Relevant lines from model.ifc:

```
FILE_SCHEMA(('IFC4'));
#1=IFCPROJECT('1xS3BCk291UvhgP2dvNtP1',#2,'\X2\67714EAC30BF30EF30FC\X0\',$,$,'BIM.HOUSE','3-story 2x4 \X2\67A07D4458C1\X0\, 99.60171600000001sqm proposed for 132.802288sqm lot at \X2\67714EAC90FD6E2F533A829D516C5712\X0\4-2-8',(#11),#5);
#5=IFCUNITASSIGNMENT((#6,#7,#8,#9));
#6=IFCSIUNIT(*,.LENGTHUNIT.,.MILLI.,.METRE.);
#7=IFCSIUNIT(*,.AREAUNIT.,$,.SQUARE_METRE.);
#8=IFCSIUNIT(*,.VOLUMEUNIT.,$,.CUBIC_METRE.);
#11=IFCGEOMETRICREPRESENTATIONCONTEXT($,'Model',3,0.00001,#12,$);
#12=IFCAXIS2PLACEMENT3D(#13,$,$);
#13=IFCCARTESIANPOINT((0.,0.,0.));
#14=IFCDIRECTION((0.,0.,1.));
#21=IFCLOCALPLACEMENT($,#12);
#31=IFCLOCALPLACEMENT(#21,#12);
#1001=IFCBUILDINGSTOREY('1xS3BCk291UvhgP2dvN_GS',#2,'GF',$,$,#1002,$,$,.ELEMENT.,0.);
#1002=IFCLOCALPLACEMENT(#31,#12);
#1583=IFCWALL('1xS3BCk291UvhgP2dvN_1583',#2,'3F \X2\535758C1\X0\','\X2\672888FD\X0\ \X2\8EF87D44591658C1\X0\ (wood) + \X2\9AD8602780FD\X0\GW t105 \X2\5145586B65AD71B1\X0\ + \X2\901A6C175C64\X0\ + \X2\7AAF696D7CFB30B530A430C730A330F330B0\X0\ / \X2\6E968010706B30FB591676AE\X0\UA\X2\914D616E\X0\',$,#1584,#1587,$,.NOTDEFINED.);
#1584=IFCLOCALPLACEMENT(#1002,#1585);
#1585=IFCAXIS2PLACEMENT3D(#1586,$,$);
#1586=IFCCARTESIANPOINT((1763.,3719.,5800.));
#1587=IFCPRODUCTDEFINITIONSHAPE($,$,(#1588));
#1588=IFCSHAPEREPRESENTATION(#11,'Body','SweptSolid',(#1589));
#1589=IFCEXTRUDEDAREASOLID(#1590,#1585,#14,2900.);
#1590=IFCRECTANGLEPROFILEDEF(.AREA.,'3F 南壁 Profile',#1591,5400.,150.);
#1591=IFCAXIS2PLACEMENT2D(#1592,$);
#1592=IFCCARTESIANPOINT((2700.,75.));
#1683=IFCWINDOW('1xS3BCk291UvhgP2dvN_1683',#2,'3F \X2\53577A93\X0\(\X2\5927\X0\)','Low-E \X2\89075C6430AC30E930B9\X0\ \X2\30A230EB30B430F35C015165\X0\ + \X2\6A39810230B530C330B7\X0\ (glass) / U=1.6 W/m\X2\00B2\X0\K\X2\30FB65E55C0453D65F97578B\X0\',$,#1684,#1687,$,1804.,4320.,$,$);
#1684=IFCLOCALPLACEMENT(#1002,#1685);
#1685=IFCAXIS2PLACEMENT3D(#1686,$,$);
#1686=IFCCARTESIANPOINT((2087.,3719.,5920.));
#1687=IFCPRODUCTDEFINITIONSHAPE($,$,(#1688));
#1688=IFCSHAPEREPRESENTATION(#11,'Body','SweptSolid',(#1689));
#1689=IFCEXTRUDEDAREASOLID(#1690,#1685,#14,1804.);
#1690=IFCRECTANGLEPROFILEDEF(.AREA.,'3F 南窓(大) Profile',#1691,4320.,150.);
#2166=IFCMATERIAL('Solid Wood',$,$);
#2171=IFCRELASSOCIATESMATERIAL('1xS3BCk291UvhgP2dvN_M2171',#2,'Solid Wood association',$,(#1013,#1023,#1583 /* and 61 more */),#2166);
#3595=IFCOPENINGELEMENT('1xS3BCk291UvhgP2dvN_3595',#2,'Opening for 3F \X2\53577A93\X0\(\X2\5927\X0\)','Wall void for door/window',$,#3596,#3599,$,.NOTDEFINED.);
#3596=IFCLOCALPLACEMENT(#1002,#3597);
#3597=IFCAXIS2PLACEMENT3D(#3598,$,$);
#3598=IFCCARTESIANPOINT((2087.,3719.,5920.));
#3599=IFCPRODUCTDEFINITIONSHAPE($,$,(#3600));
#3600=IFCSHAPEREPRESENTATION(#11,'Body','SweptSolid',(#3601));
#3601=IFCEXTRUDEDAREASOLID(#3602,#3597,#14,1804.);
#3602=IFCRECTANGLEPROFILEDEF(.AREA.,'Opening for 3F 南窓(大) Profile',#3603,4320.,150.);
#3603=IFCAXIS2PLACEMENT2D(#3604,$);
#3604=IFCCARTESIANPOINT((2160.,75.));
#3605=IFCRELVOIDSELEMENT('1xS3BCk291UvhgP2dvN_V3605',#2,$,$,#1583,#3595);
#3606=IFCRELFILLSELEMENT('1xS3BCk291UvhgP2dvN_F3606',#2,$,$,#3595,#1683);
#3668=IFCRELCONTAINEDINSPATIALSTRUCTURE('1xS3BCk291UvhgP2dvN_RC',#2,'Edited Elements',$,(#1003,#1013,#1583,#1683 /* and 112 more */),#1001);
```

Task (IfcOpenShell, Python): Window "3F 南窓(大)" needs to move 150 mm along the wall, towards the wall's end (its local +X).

```python
import ifcopenshell
import ifcopenshell.api.geometry
import ifcopenshell.util.placement
import ifcopenshell.util.unit

model = ifcopenshell.open("model.ifc")
unit_scale = ifcopenshell.util.unit.calculate_unit_scale(model)

window = model.by_guid("1xS3BCk291UvhgP2dvN_1683")
opening = window.FillsVoids[0].RelatingOpeningElement
wall = opening.VoidsElements[0].RelatingBuildingElement

wall_matrix = ifcopenshell.util.placement.get_local_placement(wall.ObjectPlacement)
shift = wall_matrix[:3, 0] * 0.15 / unit_scale
before = ifcopenshell.util.placement.get_local_placement(window.ObjectPlacement)[:3, 3].copy()

# The window is not placed relative to its opening, so move both.
for product in (opening, window):
    matrix = ifcopenshell.util.placement.get_local_placement(product.ObjectPlacement)
    matrix[:3, 3] += shift
    ifcopenshell.api.geometry.edit_object_placement(model, product=product, matrix=matrix, is_si=False)

after = ifcopenshell.util.placement.get_local_placement(window.ObjectPlacement)[:3, 3]
print("window moved by", (after - before).round(3) + 0.0)

model.write("model_edited.ifc")
```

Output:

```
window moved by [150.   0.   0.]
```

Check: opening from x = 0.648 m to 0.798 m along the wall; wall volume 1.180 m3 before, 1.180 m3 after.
